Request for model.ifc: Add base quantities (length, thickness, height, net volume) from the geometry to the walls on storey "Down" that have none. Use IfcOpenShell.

First a look at what the model holds.

```python
import ifcopenshell
import ifcopenshell.util.element
import ifcopenshell.util.unit

model = ifcopenshell.open("model.ifc")
print(model.schema)
for unit_type in ("LENGTHUNIT", "AREAUNIT", "VOLUMEUNIT"):
    print(unit_type, ifcopenshell.util.unit.calculate_unit_scale(model, unit_type))
storey = next(s for s in model.by_type("IfcBuildingStorey") if s.Name == "Down")
walls = [e for e in ifcopenshell.util.element.get_decomposition(storey) if e.is_a("IfcWall")]
for e in sorted(walls, key=lambda e: e.id()):
    print(e.id(), e.is_a(), e.Name, list(ifcopenshell.util.element.get_psets(e, qtos_only=True)), sep=" | ")
```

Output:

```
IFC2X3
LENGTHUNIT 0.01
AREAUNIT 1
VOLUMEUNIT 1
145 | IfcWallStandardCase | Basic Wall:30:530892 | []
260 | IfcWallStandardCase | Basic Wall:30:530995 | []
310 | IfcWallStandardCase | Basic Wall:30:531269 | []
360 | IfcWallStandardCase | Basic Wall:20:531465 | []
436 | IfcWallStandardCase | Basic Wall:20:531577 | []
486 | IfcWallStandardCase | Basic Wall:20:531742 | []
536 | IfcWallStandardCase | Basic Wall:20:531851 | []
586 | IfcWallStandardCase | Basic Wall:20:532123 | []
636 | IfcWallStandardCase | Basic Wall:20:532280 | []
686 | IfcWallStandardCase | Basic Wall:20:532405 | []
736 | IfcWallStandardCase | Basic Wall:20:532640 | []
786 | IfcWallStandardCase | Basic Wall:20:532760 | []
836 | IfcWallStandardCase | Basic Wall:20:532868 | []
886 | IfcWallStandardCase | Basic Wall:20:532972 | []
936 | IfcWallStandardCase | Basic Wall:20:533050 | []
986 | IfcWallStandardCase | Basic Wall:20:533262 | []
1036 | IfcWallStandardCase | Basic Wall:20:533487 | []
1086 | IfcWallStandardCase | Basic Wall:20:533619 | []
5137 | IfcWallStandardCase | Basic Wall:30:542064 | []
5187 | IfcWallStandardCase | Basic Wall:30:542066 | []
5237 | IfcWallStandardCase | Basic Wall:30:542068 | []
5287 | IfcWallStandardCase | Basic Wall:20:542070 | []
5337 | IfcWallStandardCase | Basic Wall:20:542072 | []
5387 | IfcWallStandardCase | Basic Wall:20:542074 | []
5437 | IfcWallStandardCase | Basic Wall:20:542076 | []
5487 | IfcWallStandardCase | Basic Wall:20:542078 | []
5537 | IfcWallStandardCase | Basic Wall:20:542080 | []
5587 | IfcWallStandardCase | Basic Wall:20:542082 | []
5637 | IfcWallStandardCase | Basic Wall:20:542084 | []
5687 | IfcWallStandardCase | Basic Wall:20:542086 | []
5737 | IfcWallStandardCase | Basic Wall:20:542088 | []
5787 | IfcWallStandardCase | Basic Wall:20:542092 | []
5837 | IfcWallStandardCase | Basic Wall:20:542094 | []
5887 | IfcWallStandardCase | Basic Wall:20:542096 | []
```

```python
import ifcopenshell
import ifcopenshell.api.pset
import ifcopenshell.geom
import ifcopenshell.util.element
import ifcopenshell.util.shape
import ifcopenshell.util.unit

model = ifcopenshell.open("model.ifc")
unit_scale = ifcopenshell.util.unit.calculate_unit_scale(model)
volume_scale = ifcopenshell.util.unit.calculate_unit_scale(model, "VOLUMEUNIT")
settings = ifcopenshell.geom.settings()

storey = next(s for s in model.by_type("IfcBuildingStorey") if s.Name == "Down")
walls = [e for e in ifcopenshell.util.element.get_decomposition(storey) if e.is_a("IfcWall")]

for e in sorted(walls, key=lambda e: e.id()):
    if ifcopenshell.util.element.get_psets(e, qtos_only=True, should_inherit=False):
        continue
    # Geometry comes back in metres, in the element's own axes.
    shape = ifcopenshell.geom.create_shape(settings, e)
    values = {
        "Length": ifcopenshell.util.shape.get_x(shape.geometry) / unit_scale,
        "Width": ifcopenshell.util.shape.get_y(shape.geometry) / unit_scale,
        "Height": ifcopenshell.util.shape.get_z(shape.geometry) / unit_scale,
        "NetVolume": ifcopenshell.util.shape.get_volume(shape.geometry) / volume_scale,
    }
    qto = ifcopenshell.api.pset.add_qto(model, product=e, name="BaseQuantities")
    ifcopenshell.api.pset.edit_qto(model, qto=qto, properties=values)
    print(e.id(), {k: round(v, 3) for k, v in values.items()})

model.write("model_edited.ifc")
```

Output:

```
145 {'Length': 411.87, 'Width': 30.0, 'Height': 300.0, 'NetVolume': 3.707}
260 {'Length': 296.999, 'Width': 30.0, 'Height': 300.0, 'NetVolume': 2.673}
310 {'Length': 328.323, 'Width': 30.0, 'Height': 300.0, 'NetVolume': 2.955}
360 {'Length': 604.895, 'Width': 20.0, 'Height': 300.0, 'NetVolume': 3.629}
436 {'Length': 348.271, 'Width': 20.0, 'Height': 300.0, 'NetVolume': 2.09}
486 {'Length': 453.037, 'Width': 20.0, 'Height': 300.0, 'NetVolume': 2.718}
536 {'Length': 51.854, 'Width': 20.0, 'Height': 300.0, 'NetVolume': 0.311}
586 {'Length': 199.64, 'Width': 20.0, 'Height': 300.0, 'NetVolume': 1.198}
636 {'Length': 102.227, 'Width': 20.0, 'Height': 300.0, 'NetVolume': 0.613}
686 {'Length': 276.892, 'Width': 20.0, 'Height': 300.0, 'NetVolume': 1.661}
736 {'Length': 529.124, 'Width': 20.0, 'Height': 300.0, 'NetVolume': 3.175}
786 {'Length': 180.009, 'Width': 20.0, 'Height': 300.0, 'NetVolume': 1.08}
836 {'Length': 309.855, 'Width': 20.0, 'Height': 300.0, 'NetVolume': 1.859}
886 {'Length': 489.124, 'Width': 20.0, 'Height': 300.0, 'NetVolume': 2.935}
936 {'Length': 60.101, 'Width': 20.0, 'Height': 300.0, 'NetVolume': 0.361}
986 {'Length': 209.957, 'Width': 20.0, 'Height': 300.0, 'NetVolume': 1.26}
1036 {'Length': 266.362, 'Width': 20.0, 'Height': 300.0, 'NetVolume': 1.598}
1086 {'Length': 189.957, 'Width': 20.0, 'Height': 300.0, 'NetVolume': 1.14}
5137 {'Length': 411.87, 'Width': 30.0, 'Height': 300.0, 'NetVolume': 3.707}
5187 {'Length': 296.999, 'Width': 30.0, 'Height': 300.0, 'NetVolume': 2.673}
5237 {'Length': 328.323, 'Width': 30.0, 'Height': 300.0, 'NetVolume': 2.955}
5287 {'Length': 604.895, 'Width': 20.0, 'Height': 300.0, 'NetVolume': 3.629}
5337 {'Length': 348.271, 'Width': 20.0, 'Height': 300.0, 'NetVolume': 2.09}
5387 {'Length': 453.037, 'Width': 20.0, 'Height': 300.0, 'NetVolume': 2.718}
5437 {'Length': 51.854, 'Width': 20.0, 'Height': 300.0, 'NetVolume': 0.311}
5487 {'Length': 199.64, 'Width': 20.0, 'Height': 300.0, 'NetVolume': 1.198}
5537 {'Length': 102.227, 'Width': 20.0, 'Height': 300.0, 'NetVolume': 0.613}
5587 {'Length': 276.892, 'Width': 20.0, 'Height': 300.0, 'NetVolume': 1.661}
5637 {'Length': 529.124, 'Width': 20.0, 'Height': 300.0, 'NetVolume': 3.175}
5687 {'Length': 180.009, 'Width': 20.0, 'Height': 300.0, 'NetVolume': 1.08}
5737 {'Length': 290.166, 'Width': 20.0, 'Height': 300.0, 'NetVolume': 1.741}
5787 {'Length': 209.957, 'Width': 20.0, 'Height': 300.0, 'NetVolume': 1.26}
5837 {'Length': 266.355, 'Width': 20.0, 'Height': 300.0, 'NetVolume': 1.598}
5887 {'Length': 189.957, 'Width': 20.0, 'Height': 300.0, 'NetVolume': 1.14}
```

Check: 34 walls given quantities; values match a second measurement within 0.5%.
